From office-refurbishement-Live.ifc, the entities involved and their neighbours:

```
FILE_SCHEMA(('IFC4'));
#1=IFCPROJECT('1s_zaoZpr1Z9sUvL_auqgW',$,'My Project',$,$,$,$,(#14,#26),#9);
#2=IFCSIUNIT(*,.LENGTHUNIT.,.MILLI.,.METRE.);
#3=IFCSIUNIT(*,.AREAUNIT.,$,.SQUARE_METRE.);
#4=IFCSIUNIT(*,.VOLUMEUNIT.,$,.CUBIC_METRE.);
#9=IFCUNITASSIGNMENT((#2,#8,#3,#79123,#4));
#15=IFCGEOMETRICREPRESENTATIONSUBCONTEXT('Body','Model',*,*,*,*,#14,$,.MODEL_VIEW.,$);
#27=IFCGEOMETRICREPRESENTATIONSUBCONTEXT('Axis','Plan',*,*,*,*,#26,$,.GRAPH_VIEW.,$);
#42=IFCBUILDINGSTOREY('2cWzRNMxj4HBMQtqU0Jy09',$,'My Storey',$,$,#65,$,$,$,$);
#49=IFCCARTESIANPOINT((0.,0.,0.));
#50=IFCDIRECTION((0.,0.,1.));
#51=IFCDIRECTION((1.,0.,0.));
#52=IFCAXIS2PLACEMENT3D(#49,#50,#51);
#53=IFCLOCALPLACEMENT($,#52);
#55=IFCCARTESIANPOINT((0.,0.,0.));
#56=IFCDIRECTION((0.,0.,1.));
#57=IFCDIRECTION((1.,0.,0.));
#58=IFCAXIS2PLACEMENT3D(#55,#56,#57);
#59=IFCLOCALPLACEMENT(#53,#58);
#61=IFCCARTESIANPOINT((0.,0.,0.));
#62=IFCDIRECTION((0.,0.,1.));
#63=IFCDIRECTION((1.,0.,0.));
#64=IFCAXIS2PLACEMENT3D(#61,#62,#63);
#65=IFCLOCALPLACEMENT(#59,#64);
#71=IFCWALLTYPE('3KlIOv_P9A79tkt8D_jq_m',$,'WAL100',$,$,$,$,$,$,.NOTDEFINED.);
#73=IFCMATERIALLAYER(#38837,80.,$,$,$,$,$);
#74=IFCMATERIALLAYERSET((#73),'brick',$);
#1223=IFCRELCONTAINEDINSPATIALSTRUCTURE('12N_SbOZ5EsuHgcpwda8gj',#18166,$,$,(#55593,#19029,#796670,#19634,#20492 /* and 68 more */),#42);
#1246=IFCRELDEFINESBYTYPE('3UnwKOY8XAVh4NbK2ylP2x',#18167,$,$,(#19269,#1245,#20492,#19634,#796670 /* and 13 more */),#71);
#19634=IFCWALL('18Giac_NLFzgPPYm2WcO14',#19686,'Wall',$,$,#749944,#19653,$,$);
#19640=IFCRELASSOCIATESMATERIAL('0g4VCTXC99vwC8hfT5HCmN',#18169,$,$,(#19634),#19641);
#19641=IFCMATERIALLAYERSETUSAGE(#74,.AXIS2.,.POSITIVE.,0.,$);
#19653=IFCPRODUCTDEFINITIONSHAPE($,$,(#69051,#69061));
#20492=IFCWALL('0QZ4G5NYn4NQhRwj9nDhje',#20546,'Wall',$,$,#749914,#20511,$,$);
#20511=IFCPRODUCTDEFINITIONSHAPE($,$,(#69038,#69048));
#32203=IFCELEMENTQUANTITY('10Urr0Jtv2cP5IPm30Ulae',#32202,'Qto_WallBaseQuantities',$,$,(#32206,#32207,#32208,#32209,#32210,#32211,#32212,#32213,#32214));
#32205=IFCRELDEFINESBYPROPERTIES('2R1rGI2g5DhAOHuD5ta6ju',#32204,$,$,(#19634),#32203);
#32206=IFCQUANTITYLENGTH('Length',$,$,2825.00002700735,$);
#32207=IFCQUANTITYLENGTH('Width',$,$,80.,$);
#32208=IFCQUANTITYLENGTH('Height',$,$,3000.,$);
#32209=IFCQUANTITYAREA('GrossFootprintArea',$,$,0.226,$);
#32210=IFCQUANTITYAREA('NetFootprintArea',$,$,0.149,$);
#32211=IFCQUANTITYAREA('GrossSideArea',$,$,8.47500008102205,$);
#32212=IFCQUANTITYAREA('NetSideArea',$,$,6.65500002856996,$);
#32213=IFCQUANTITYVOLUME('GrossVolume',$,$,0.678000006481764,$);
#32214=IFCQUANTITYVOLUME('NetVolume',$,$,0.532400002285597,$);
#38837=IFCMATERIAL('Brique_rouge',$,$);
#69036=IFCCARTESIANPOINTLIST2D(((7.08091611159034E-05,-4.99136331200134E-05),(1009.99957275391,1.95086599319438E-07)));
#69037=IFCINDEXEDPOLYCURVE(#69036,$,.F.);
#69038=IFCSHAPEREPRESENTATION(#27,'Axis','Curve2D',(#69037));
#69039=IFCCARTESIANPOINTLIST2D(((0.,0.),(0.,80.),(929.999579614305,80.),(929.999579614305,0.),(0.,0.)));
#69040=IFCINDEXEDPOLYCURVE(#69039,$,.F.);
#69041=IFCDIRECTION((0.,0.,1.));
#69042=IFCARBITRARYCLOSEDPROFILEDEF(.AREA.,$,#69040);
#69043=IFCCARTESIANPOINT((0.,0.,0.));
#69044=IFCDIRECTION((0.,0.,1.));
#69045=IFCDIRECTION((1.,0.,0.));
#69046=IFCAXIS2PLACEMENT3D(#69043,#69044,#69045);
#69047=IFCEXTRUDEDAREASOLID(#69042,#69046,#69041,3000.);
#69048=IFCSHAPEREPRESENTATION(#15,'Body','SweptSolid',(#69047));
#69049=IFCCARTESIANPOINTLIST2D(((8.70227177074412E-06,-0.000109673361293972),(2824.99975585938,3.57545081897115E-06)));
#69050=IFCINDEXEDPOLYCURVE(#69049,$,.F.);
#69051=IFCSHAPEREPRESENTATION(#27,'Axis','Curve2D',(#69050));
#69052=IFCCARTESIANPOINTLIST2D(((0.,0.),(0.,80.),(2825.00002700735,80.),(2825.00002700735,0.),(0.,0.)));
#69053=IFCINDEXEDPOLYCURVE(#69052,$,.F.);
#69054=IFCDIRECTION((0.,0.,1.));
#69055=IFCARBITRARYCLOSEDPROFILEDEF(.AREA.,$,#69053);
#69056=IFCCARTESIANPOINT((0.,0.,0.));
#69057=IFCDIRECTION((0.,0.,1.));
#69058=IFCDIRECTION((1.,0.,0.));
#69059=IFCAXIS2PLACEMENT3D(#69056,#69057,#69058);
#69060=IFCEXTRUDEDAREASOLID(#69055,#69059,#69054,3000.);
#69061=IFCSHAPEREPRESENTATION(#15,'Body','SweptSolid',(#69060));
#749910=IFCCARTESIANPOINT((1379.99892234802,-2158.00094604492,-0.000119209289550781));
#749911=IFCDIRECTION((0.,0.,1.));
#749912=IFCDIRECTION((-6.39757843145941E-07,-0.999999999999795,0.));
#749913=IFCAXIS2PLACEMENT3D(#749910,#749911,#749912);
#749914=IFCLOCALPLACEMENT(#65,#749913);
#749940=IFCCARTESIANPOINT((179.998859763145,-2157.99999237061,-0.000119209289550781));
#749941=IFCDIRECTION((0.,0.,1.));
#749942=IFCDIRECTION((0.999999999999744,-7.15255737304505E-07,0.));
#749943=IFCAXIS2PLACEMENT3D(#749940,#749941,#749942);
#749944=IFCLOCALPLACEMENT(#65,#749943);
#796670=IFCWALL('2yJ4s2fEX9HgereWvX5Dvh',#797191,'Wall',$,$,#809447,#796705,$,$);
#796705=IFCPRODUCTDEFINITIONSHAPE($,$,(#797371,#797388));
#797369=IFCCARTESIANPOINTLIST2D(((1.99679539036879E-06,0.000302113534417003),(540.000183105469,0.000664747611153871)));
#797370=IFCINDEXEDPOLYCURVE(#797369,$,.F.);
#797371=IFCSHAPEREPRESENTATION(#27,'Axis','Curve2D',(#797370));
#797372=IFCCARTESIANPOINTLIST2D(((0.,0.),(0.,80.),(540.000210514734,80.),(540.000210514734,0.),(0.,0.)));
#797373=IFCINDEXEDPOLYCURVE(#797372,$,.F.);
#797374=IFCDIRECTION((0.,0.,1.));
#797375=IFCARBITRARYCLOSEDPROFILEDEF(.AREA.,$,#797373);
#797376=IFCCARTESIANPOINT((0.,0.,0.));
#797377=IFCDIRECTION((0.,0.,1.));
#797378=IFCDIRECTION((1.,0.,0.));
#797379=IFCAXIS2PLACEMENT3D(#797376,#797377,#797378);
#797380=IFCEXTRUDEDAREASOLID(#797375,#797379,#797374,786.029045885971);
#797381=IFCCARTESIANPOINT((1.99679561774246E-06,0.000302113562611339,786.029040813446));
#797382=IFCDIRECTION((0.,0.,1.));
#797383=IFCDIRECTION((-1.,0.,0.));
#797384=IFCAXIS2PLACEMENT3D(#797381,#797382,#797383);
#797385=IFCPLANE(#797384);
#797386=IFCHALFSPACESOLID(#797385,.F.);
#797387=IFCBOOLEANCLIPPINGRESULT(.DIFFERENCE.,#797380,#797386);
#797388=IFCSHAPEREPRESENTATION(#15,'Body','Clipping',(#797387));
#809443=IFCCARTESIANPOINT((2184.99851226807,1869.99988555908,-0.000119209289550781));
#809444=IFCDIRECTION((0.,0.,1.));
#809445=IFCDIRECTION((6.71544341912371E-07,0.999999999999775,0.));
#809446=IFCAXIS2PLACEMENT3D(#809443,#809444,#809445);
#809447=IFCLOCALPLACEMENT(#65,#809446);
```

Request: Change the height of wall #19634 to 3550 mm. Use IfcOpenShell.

```python
import ifcopenshell
import ifcopenshell.api.pset
import ifcopenshell.geom
import ifcopenshell.util.element
import ifcopenshell.util.representation
import ifcopenshell.util.shape
import ifcopenshell.util.unit

model = ifcopenshell.open("office-refurbishement-Live.ifc")
unit_scale = ifcopenshell.util.unit.calculate_unit_scale(model)
area_scale = ifcopenshell.util.unit.calculate_unit_scale(model, "AREAUNIT")
volume_scale = ifcopenshell.util.unit.calculate_unit_scale(model, "VOLUMEUNIT")
settings = ifcopenshell.geom.settings()


def volume(element):
    """Net volume in cubic metres, openings subtracted."""
    shape = ifcopenshell.geom.create_shape(settings, element)
    return ifcopenshell.util.shape.get_volume(shape.geometry)


wall = model.by_guid("18Giac_NLFzgPPYm2WcO14")
before = volume(wall)

body = ifcopenshell.util.representation.get_representation(wall, "Model", "Body")
solid = body.Items[0]
old_height = solid.Depth
solid.Depth = 3.55 / unit_scale
after = volume(wall)
thickness = 0.08  # wall thickness in metres

# Update the stored height, areas and volumes.
qto = model.by_id(ifcopenshell.util.element.get_pset(wall, "Qto_WallBaseQuantities", should_inherit=False)["id"])
ifcopenshell.api.pset.edit_qto(model, qto=qto, properties={
    "Height": solid.Depth,
    "GrossSideArea": ifcopenshell.util.element.get_pset(wall, "Qto_WallBaseQuantities", "GrossSideArea") * solid.Depth / old_height,
    "NetSideArea": after / thickness / area_scale,
    "GrossVolume": ifcopenshell.util.element.get_pset(wall, "Qto_WallBaseQuantities", "GrossVolume") * solid.Depth / old_height,
    "NetVolume": after / volume_scale,
})

print(f"height {old_height:g} -> {solid.Depth:g}, volume {before:.3f} -> {after:.3f} m3")

model.write("office-refurbishement-Live_rev.ifc")
```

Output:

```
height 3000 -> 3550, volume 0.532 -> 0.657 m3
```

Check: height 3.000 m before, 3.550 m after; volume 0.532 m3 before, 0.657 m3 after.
